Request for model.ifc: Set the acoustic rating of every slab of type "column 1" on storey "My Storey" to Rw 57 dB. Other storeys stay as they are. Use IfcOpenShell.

First a look at what the model holds.

```python
import ifcopenshell
import ifcopenshell.util.element

model = ifcopenshell.open("model.ifc")
print(model.schema)
storey = next(s for s in model.by_type("IfcBuildingStorey") if s.Name == "My Storey")
slabs = [e for e in ifcopenshell.util.element.get_decomposition(storey) if e.is_a("IfcSlab")]
seen = {}
for e in slabs:
    element_type = ifcopenshell.util.element.get_type(e)
    key = (element_type.Name if element_type != e and element_type else None, ifcopenshell.util.element.get_pset(e, "Pset_SlabCommon", "AcousticRating"))
    seen[key] = seen.get(key, 0) + 1
for (name, value), count in sorted(seen.items(), key=str):
    print(count, "x", name, "|", value)
```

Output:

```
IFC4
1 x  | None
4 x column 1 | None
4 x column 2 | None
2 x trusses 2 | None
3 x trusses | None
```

```python
import ifcopenshell
import ifcopenshell.api.pset
import ifcopenshell.util.element

model = ifcopenshell.open("model.ifc")

storey = next(s for s in model.by_type("IfcBuildingStorey") if s.Name == "My Storey")
slabs = [e for e in ifcopenshell.util.element.get_decomposition(storey) if e.is_a("IfcSlab")]

count = 0
for e in slabs:
    element_type = ifcopenshell.util.element.get_type(e)
    if element_type in (None, e) or element_type.Name != "column 1":
        continue
    # add_pset returns the element's existing set when there is one.
    pset = ifcopenshell.api.pset.add_pset(model, product=e, name="Pset_SlabCommon")
    ifcopenshell.api.pset.edit_pset(model, pset=pset, properties={"AcousticRating": "Rw 57 dB"})
    count += 1

print(count, "slabs updated")

model.write("model_v2.ifc")
```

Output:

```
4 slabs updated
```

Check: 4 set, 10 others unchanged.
